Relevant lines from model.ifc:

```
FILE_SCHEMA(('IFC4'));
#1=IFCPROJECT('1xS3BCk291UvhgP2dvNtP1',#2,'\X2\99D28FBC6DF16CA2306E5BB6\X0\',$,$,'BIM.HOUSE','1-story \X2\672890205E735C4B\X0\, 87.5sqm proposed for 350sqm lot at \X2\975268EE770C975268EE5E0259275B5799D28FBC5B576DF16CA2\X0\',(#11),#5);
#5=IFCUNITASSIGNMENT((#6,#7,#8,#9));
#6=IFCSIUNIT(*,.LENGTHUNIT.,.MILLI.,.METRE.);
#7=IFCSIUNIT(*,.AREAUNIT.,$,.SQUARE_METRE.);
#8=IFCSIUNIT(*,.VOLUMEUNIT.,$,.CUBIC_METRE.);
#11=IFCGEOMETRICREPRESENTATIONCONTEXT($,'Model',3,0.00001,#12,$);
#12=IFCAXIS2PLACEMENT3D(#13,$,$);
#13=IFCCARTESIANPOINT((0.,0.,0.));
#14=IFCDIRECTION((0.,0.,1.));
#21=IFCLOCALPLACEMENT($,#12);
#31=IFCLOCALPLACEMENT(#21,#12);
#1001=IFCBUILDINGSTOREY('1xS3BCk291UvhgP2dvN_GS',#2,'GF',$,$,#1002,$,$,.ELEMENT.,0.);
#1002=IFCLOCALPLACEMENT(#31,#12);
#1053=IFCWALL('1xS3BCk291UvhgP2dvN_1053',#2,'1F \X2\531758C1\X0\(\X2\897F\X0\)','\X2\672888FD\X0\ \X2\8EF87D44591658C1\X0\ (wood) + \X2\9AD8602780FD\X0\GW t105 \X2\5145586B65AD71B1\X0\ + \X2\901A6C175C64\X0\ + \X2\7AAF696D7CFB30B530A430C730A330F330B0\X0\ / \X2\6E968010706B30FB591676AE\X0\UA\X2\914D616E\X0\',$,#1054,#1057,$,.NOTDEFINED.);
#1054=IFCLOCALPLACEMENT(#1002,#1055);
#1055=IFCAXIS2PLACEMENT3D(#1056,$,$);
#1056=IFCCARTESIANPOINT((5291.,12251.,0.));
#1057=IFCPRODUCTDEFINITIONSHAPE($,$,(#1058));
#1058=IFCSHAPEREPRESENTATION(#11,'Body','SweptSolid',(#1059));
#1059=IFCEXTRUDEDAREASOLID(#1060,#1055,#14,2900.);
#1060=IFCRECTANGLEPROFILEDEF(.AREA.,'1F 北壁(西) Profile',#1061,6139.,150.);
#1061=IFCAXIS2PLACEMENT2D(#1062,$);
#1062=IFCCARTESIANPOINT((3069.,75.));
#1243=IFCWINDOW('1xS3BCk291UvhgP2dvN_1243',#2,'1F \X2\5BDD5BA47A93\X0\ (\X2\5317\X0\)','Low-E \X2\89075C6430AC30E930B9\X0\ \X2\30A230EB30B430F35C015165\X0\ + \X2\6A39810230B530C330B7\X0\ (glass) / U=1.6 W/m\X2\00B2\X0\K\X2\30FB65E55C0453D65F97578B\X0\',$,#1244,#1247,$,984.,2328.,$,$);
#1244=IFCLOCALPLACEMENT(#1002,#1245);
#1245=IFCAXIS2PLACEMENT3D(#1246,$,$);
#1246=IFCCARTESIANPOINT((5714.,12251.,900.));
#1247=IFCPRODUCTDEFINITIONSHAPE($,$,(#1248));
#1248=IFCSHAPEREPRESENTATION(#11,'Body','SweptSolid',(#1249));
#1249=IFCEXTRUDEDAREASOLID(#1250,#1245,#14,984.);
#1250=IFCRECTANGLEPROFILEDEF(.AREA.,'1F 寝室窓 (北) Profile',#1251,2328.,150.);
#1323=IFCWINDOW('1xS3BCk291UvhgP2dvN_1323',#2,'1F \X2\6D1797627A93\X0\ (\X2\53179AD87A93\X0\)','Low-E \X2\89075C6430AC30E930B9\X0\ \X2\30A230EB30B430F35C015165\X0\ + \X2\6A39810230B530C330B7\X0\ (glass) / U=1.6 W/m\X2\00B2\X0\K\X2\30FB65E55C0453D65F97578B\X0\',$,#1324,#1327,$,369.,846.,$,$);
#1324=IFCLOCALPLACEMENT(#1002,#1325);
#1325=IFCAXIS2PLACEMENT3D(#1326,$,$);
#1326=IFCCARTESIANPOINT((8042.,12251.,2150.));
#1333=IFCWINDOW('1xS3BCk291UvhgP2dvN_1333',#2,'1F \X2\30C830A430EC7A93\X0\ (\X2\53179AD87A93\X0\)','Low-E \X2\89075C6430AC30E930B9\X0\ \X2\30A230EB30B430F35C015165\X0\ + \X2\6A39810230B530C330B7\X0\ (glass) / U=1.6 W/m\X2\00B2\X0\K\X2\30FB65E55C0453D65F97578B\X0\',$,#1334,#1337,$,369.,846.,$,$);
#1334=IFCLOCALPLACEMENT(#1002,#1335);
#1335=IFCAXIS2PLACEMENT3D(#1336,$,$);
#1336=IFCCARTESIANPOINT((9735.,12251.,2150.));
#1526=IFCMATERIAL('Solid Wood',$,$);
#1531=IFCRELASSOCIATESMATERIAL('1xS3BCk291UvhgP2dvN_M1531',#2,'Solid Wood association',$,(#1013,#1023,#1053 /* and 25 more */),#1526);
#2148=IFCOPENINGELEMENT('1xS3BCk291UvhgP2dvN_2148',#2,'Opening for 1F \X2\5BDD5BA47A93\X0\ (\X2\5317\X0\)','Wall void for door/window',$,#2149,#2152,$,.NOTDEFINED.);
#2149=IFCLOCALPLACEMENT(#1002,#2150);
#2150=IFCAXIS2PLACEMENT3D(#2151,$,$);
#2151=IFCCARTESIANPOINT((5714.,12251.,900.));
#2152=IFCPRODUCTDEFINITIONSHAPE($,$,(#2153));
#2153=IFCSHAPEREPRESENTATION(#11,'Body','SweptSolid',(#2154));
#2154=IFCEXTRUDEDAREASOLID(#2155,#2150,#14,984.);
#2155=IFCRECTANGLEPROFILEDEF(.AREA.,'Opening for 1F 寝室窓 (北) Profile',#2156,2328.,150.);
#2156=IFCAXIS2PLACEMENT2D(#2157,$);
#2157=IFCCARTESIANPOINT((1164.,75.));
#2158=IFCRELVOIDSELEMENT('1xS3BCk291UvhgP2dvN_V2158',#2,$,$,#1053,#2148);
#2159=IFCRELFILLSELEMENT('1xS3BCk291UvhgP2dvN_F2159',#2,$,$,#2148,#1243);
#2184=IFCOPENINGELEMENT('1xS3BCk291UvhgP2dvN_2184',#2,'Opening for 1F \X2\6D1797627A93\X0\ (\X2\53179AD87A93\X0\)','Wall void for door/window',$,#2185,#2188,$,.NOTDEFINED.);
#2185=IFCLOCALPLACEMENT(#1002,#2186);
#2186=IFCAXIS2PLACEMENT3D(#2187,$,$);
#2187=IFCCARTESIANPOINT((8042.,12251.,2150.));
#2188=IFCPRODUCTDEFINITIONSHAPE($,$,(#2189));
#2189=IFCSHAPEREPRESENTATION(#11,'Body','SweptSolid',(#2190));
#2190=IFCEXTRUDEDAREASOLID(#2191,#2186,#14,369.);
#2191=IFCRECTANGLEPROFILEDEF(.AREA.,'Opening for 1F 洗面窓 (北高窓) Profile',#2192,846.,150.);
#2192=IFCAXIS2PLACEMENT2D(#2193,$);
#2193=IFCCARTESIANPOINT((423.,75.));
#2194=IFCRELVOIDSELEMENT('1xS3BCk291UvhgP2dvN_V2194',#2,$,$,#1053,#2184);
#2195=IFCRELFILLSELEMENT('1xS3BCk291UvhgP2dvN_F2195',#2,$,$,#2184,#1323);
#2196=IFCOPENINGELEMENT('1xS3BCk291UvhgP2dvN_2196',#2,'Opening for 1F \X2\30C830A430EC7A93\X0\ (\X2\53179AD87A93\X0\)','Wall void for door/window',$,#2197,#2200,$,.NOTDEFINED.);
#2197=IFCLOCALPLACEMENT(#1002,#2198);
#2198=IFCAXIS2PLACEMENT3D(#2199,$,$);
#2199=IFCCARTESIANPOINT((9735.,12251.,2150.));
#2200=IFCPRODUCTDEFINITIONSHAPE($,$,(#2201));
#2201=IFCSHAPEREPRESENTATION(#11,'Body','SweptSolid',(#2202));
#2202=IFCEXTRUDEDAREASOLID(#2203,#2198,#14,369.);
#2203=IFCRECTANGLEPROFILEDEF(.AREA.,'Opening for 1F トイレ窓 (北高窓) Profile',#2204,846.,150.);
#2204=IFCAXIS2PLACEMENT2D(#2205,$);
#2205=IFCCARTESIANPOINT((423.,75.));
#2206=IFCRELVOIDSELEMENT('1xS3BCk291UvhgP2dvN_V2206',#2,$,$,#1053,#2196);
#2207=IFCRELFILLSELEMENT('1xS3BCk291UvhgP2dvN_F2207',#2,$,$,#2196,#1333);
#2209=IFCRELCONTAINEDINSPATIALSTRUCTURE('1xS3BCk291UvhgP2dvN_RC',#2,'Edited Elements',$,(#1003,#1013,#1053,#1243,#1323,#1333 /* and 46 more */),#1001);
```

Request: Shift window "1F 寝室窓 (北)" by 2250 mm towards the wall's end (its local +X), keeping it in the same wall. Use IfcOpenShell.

```python
import ifcopenshell
import ifcopenshell.api.geometry
import ifcopenshell.util.placement

model = ifcopenshell.open("model.ifc")

window = model.by_guid("1xS3BCk291UvhgP2dvN_1243")
opening = window.FillsVoids[0].RelatingOpeningElement
wall = opening.VoidsElements[0].RelatingBuildingElement

wall_matrix = ifcopenshell.util.placement.get_local_placement(wall.ObjectPlacement)
shift = wall_matrix[:3, 0] * 2250.0
before = ifcopenshell.util.placement.get_local_placement(window.ObjectPlacement)[:3, 3].copy()

# The window is not placed relative to its opening, so move both.
for product in (opening, window):
    matrix = ifcopenshell.util.placement.get_local_placement(product.ObjectPlacement)
    matrix[:3, 3] += shift
    ifcopenshell.api.geometry.edit_object_placement(model, product=product, matrix=matrix, is_si=False)

after = ifcopenshell.util.placement.get_local_placement(window.ObjectPlacement)[:3, 3]
print("window moved by", (after - before).round(3) + 0.0)

model.write("model_edited.ifc")
```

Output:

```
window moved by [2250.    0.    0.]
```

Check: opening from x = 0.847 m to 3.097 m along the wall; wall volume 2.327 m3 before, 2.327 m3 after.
